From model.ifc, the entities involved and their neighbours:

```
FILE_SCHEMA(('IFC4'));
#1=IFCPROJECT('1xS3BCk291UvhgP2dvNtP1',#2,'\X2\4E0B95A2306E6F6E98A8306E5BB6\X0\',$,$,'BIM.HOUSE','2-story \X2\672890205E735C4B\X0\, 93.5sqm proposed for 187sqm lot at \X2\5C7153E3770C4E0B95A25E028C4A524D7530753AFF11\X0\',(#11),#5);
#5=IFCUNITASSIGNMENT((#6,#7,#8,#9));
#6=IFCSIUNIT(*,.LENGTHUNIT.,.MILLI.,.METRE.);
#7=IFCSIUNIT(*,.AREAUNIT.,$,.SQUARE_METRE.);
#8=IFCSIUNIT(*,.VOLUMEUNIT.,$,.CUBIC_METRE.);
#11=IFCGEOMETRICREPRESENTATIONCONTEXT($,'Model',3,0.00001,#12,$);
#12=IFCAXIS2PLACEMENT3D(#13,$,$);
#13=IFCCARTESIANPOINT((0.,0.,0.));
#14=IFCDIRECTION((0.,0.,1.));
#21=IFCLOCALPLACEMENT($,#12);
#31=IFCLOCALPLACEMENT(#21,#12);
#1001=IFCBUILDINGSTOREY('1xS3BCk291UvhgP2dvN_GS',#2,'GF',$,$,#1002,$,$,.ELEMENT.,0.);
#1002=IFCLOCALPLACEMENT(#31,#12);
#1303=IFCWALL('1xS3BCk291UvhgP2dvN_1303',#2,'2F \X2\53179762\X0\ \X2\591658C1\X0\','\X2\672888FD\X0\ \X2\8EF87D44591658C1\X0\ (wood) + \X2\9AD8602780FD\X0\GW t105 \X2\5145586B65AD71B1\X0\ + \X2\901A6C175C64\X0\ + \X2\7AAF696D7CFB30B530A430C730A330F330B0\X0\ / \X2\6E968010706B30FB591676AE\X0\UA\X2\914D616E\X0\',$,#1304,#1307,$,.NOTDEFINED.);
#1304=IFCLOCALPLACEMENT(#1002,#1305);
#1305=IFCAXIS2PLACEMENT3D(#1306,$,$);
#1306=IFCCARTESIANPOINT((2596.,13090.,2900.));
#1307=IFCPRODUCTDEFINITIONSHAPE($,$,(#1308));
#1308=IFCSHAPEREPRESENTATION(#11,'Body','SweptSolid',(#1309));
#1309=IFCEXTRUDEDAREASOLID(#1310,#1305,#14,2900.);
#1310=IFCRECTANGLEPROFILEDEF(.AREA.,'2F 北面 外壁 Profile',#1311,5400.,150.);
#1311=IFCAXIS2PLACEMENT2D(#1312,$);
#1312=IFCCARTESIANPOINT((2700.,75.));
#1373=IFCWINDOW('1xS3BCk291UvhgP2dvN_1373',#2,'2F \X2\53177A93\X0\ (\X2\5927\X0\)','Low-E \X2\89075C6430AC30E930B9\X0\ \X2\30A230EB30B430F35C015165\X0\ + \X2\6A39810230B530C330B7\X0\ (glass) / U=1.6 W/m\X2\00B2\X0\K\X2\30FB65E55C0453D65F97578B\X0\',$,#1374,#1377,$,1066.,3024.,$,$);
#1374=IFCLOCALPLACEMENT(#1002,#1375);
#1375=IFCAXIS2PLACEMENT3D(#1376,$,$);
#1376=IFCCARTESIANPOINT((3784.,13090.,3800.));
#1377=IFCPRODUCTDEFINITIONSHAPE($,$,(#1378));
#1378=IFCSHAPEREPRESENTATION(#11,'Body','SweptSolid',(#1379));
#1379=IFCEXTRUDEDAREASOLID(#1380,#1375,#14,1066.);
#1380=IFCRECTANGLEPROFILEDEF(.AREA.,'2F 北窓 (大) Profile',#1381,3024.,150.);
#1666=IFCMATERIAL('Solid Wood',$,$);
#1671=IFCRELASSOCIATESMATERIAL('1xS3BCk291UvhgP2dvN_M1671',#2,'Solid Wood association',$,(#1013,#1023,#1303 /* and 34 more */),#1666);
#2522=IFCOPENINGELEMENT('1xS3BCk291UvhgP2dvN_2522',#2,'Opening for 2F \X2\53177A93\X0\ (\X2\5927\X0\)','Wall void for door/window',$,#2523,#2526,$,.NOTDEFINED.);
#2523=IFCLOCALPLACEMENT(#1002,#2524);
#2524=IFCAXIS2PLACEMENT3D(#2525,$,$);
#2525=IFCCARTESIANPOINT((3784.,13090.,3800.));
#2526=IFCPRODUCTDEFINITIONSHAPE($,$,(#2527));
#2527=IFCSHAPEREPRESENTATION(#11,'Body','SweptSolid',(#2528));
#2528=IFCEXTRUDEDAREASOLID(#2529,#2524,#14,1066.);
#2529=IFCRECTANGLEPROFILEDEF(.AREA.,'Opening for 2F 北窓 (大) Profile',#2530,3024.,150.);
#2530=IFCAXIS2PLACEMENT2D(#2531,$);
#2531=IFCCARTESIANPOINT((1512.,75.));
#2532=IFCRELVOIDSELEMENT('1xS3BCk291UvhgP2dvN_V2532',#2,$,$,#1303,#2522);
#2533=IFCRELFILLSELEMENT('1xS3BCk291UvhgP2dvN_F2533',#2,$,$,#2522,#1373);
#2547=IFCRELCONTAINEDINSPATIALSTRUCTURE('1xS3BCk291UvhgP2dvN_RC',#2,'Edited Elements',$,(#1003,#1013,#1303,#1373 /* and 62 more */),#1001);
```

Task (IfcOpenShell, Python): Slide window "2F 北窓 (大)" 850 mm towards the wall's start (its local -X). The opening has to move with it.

```python
import ifcopenshell
import ifcopenshell.api.geometry
import ifcopenshell.util.placement
import ifcopenshell.util.unit

model = ifcopenshell.open("model.ifc")
unit_scale = ifcopenshell.util.unit.calculate_unit_scale(model)

window = model.by_guid("1xS3BCk291UvhgP2dvN_1373")
opening = window.FillsVoids[0].RelatingOpeningElement
wall = opening.VoidsElements[0].RelatingBuildingElement

wall_matrix = ifcopenshell.util.placement.get_local_placement(wall.ObjectPlacement)
shift = wall_matrix[:3, 0] * -0.85 / unit_scale
before = ifcopenshell.util.placement.get_local_placement(window.ObjectPlacement)[:3, 3].copy()

# The window is not placed relative to its opening, so move both.
for product in (opening, window):
    matrix = ifcopenshell.util.placement.get_local_placement(product.ObjectPlacement)
    matrix[:3, 3] += shift
    ifcopenshell.api.geometry.edit_object_placement(model, product=product, matrix=matrix, is_si=False)

after = ifcopenshell.util.placement.get_local_placement(window.ObjectPlacement)[:3, 3]
print("window moved by", (after - before).round(3) + 0.0)

model.write("model_rev.ifc")
```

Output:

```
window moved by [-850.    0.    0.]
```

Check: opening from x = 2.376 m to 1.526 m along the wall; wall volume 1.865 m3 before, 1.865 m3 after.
